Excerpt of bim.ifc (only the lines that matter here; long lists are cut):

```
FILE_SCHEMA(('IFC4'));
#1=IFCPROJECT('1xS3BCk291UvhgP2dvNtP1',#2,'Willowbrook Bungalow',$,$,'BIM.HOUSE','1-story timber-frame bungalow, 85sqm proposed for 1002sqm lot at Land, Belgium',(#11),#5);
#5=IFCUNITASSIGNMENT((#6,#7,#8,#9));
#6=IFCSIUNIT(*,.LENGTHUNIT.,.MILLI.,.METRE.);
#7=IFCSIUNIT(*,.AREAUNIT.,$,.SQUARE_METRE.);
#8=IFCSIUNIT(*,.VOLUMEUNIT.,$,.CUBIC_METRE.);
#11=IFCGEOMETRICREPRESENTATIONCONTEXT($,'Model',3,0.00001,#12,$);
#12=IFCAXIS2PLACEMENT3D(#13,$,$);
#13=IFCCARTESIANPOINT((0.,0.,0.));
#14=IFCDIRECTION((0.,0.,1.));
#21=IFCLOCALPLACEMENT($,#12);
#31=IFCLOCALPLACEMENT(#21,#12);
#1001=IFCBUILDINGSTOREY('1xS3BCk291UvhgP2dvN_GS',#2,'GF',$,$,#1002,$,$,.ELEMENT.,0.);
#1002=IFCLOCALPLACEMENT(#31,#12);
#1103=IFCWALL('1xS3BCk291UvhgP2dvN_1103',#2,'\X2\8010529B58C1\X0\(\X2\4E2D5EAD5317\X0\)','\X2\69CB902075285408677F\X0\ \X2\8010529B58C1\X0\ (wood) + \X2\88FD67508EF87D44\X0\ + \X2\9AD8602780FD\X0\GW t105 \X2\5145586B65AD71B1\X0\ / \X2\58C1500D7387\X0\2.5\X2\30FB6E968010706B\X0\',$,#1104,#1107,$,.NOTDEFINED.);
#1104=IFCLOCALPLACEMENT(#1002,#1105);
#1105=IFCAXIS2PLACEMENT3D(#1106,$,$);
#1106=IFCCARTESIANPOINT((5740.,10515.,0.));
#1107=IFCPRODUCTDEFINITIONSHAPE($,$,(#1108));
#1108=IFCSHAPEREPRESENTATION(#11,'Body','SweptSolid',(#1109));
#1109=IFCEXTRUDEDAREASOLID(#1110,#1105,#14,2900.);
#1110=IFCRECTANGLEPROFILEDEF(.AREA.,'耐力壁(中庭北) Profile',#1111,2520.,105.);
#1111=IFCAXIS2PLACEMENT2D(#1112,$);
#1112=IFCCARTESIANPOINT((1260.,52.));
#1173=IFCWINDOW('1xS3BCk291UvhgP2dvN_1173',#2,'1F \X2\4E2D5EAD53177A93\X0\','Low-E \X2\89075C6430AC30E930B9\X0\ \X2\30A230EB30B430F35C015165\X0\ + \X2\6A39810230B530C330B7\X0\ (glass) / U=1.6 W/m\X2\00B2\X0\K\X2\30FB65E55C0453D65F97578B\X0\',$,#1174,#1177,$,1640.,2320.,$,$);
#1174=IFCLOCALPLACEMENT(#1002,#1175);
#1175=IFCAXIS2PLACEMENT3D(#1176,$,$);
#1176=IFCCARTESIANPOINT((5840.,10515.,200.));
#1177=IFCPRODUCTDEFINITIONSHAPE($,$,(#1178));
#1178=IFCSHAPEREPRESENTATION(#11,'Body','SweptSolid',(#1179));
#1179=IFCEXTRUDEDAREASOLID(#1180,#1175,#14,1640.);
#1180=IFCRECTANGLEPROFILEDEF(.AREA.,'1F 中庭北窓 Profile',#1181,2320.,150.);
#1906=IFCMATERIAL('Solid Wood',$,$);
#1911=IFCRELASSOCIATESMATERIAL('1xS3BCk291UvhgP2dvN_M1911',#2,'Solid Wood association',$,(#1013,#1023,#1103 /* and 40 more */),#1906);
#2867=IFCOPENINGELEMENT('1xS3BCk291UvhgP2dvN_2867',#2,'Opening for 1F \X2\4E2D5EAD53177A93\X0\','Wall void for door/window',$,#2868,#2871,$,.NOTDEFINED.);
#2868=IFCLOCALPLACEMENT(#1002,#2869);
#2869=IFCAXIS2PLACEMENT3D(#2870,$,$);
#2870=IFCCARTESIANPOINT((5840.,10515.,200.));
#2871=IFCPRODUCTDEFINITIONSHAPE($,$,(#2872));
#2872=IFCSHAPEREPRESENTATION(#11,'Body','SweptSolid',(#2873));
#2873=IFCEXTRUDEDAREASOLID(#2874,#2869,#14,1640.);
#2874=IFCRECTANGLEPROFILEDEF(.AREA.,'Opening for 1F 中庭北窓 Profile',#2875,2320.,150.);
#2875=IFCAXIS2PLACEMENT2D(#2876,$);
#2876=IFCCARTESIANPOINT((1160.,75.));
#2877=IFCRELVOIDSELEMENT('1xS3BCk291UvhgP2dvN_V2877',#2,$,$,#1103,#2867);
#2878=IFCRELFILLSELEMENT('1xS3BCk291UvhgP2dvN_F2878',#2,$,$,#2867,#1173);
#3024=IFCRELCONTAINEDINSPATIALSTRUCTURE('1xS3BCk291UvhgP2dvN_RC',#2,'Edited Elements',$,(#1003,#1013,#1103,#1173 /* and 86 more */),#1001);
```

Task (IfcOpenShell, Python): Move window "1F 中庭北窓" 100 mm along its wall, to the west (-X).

```python
import ifcopenshell
import ifcopenshell.api.geometry
import ifcopenshell.util.placement
import ifcopenshell.util.unit

model = ifcopenshell.open("bim.ifc")
unit_scale = ifcopenshell.util.unit.calculate_unit_scale(model)

window = model.by_guid("1xS3BCk291UvhgP2dvN_1173")
opening = window.FillsVoids[0].RelatingOpeningElement
wall = opening.VoidsElements[0].RelatingBuildingElement

wall_matrix = ifcopenshell.util.placement.get_local_placement(wall.ObjectPlacement)
shift = wall_matrix[:3, 0] * -0.1 / unit_scale
before = ifcopenshell.util.placement.get_local_placement(window.ObjectPlacement)[:3, 3].copy()

# The window is not placed relative to its opening, so move both.
for product in (opening, window):
    matrix = ifcopenshell.util.placement.get_local_placement(product.ObjectPlacement)
    matrix[:3, 3] += shift
    ifcopenshell.api.geometry.edit_object_placement(model, product=product, matrix=matrix, is_si=False)

after = ifcopenshell.util.placement.get_local_placement(window.ObjectPlacement)[:3, 3]
print("window moved by", (after - before).round(3) + 0.0)

model.write("bim_edited.ifc")
```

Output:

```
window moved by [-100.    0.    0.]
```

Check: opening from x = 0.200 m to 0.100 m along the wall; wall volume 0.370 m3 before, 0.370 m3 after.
